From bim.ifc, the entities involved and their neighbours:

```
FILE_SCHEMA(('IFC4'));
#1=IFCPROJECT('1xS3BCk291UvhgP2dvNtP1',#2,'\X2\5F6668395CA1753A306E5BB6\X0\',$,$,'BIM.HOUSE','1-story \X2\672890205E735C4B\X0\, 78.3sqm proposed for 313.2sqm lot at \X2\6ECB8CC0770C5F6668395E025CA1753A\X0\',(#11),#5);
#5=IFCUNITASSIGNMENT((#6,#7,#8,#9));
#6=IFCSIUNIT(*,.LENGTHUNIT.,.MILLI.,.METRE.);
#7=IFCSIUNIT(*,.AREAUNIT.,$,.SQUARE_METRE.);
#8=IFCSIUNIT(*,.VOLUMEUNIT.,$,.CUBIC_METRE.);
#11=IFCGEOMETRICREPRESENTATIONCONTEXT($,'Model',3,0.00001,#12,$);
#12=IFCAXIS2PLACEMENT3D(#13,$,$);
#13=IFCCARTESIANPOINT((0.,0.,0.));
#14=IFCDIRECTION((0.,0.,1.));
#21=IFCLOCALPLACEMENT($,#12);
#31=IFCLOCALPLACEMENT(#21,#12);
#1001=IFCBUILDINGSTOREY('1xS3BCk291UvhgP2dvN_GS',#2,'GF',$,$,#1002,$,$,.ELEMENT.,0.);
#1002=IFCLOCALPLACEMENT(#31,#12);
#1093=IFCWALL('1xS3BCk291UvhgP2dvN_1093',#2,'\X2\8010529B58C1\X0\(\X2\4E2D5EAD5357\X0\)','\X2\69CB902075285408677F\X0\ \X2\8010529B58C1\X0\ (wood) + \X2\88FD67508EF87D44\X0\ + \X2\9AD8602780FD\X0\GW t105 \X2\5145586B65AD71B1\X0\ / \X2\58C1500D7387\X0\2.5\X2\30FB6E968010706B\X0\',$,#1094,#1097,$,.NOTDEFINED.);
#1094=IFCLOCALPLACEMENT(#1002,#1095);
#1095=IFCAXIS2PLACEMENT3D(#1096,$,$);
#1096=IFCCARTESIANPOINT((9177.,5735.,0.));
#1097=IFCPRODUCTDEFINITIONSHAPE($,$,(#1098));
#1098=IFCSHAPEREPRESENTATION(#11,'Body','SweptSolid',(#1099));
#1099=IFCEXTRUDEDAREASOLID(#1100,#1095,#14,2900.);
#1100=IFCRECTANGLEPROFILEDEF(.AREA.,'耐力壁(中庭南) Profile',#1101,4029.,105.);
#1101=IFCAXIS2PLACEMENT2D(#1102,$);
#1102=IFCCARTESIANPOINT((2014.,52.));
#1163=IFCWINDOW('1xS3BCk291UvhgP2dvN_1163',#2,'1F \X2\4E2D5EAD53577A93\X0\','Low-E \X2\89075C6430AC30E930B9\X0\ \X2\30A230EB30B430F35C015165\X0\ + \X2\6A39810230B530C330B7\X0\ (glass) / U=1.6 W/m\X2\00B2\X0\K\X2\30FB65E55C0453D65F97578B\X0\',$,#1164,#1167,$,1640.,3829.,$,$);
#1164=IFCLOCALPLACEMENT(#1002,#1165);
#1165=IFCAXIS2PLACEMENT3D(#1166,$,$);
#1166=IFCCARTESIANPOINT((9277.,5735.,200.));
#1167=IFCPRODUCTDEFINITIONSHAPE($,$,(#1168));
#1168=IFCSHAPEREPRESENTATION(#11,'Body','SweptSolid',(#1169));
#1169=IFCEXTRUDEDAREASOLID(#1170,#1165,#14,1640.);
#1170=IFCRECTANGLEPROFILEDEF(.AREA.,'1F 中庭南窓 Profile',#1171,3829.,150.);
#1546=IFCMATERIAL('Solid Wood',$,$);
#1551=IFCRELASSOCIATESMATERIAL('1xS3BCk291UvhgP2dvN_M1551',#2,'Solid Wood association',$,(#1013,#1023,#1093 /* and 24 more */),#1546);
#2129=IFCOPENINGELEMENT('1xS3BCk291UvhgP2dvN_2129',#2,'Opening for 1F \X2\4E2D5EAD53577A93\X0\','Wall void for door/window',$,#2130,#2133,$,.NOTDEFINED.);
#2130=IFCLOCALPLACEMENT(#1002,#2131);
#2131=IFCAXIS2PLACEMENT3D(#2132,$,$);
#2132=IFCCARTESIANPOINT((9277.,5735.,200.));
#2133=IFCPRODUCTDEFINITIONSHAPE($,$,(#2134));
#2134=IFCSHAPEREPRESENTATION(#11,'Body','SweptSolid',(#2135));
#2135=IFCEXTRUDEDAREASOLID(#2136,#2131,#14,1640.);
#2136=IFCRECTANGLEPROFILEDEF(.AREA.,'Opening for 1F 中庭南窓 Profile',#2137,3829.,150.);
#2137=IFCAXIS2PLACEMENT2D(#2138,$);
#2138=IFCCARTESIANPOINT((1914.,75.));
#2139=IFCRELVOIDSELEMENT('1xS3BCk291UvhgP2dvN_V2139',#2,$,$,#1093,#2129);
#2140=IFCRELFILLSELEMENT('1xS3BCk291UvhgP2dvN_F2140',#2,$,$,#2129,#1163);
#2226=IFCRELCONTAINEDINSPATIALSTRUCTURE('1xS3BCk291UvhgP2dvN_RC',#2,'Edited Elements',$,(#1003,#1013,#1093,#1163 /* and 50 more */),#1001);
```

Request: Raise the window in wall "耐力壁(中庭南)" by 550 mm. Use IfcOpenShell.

```python
import numpy as np
import ifcopenshell
import ifcopenshell.api.geometry
import ifcopenshell.util.placement
import ifcopenshell.util.unit

model = ifcopenshell.open("bim.ifc")
unit_scale = ifcopenshell.util.unit.calculate_unit_scale(model)

window = model.by_guid("1xS3BCk291UvhgP2dvN_1163")
opening = window.FillsVoids[0].RelatingOpeningElement
dz = 0.55 / unit_scale

shift = np.array([0.0, 0.0, dz])
# The window is not placed relative to its opening, so move both.
for product in (opening, window):
    matrix = ifcopenshell.util.placement.get_local_placement(product.ObjectPlacement)
    matrix[:3, 3] += shift
    ifcopenshell.api.geometry.edit_object_placement(model, product=product, matrix=matrix, is_si=False)

print(f"moved by {dz * unit_scale:+.3f} m")

model.write("bim_v2.ifc")
```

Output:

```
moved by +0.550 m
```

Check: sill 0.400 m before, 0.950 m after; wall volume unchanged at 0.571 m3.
